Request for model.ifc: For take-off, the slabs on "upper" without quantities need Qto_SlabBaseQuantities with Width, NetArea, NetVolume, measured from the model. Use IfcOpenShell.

First a look at what the model holds.

```python
import ifcopenshell
import ifcopenshell.util.element
import ifcopenshell.util.unit

model = ifcopenshell.open("model.ifc")
print(model.schema)
for unit_type in ("LENGTHUNIT", "AREAUNIT", "VOLUMEUNIT"):
    print(unit_type, ifcopenshell.util.unit.calculate_unit_scale(model, unit_type))
storey = next(s for s in model.by_type("IfcBuildingStorey") if s.Name == "upper")
slabs = [e for e in ifcopenshell.util.element.get_decomposition(storey) if e.is_a("IfcSlab")]
for e in sorted(slabs, key=lambda e: e.id()):
    print(e.id(), e.is_a(), e.Name, list(ifcopenshell.util.element.get_psets(e, qtos_only=True)), sep=" | ")
```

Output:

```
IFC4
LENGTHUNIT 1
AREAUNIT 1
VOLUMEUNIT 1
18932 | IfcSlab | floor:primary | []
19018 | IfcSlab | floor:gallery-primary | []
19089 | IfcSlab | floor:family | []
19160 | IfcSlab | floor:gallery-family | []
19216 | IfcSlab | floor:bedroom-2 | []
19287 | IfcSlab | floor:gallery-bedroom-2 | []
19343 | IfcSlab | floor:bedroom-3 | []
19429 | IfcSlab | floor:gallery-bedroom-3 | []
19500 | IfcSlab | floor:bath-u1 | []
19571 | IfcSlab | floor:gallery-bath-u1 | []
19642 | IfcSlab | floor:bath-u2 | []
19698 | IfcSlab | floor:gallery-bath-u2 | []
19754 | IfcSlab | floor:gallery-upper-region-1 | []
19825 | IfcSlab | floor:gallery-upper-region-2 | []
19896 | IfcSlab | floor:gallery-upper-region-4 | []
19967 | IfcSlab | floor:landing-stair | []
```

```python
import ifcopenshell
import ifcopenshell.api.pset
import ifcopenshell.geom
import ifcopenshell.util.element
import ifcopenshell.util.shape
import ifcopenshell.util.unit

model = ifcopenshell.open("model.ifc")
unit_scale = ifcopenshell.util.unit.calculate_unit_scale(model)
area_scale = ifcopenshell.util.unit.calculate_unit_scale(model, "AREAUNIT")
volume_scale = ifcopenshell.util.unit.calculate_unit_scale(model, "VOLUMEUNIT")
settings = ifcopenshell.geom.settings()

storey = next(s for s in model.by_type("IfcBuildingStorey") if s.Name == "upper")
slabs = [e for e in ifcopenshell.util.element.get_decomposition(storey) if e.is_a("IfcSlab")]

for e in sorted(slabs, key=lambda e: e.id()):
    if ifcopenshell.util.element.get_psets(e, qtos_only=True, should_inherit=False):
        continue
    # Geometry comes back in metres, in the element's own axes.
    shape = ifcopenshell.geom.create_shape(settings, e)
    values = {
        "Width": ifcopenshell.util.shape.get_z(shape.geometry) / unit_scale,
        "NetArea": ifcopenshell.util.shape.get_footprint_area(shape.geometry) / area_scale,
        "NetVolume": ifcopenshell.util.shape.get_volume(shape.geometry) / volume_scale,
    }
    qto = ifcopenshell.api.pset.add_qto(model, product=e, name="Qto_SlabBaseQuantities")
    ifcopenshell.api.pset.edit_qto(model, qto=qto, properties=values)
    print(e.id(), {k: round(v, 3) for k, v in values.items()})

model.write("model_v2.ifc")
```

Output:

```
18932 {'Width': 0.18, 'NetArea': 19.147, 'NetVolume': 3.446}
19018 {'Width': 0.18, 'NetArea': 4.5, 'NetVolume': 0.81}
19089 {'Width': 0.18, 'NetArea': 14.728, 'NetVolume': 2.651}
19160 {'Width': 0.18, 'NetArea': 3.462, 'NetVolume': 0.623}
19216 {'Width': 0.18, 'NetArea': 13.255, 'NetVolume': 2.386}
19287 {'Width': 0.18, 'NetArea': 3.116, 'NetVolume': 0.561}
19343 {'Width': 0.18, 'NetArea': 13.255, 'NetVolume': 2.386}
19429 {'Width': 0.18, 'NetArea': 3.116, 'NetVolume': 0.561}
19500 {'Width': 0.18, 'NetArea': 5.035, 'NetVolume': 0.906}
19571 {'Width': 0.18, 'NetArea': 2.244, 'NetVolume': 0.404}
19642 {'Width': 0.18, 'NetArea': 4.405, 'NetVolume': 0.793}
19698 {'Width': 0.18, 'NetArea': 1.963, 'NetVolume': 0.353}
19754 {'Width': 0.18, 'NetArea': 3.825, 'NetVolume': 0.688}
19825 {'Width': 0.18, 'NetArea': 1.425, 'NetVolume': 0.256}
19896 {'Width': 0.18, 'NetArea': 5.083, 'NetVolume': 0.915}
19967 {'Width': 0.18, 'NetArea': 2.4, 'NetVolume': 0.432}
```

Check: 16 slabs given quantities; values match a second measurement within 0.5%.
